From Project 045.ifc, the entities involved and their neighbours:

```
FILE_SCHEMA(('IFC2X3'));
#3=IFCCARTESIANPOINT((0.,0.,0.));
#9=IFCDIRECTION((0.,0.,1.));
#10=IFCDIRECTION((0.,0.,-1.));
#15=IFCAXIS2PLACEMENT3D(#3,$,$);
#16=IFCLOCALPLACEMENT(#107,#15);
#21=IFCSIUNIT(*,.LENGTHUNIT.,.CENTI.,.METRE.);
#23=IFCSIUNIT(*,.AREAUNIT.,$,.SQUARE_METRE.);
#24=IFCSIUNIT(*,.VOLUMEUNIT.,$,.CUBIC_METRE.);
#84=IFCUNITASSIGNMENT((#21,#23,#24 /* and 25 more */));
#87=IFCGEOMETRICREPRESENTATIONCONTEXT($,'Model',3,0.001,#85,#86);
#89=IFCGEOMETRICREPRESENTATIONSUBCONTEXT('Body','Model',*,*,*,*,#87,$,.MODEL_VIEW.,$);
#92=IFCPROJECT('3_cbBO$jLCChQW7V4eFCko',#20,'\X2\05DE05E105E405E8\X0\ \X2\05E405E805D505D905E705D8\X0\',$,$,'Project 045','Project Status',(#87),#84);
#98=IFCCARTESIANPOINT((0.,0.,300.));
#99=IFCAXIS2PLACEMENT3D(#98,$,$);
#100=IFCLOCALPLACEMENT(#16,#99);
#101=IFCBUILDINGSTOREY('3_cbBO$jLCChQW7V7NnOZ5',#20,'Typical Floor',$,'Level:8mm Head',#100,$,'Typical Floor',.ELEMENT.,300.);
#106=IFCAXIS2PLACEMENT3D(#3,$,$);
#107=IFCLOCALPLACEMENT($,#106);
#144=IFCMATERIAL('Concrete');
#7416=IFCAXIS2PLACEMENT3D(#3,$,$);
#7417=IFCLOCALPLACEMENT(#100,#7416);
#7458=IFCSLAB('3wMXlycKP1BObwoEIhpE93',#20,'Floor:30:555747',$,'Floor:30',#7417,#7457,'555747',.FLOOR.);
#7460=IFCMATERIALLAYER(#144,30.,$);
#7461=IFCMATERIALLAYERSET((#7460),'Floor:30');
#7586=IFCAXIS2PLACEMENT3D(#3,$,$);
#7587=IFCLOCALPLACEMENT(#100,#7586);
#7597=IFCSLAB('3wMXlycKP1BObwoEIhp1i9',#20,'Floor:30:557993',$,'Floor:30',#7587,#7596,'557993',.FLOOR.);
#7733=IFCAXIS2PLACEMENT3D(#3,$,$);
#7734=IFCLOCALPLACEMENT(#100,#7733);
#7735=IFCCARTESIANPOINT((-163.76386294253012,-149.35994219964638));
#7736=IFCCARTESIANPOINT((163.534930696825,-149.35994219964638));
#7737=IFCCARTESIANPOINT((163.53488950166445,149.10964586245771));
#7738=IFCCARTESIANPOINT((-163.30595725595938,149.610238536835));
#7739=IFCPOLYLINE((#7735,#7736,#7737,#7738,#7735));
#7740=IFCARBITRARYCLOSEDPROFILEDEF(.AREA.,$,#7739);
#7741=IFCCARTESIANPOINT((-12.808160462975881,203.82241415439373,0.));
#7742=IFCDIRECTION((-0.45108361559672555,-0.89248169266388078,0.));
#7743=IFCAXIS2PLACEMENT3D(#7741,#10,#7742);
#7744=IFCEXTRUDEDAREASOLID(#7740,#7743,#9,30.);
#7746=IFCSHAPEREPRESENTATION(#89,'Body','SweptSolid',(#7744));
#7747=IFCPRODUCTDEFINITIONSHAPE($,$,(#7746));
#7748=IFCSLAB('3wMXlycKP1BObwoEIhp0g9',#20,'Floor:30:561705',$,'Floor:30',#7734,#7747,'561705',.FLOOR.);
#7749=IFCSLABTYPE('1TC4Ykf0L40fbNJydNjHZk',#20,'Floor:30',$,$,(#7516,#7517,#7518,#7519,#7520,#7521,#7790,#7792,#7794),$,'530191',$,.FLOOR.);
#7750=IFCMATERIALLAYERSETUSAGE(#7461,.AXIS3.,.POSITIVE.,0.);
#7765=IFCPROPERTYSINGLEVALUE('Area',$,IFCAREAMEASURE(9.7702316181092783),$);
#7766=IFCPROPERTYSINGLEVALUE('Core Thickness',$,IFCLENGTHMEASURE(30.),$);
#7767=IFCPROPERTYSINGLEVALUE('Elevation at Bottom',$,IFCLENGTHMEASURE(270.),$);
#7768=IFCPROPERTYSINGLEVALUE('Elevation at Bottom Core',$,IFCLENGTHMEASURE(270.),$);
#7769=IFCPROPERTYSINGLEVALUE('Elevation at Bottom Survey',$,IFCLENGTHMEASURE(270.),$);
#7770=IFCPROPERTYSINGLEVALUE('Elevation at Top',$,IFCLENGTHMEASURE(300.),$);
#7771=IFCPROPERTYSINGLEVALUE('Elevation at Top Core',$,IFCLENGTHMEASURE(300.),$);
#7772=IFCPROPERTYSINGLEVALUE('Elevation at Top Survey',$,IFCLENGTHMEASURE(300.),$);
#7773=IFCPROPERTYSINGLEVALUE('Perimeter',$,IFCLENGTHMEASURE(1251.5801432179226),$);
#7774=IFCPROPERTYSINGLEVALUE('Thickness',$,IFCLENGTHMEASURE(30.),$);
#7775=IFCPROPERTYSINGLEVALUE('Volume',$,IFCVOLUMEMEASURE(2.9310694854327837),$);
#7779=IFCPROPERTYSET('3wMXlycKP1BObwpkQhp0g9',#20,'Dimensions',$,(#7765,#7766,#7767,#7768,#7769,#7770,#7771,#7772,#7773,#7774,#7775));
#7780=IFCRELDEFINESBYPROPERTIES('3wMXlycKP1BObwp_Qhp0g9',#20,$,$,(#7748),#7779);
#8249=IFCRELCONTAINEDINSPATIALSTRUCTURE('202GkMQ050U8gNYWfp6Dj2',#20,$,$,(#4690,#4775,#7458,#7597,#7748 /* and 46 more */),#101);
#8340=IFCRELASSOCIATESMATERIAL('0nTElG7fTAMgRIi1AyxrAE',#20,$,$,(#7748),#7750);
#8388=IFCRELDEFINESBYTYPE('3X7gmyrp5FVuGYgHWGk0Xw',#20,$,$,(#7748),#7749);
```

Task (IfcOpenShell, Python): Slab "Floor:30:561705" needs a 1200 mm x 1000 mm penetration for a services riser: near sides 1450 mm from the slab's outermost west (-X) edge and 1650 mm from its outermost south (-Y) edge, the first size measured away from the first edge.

```python
import numpy as np
import ifcopenshell
import ifcopenshell.api.feature
import ifcopenshell.api.geometry
import ifcopenshell.api.pset
import ifcopenshell.api.root
import ifcopenshell.geom
import ifcopenshell.util.element
import ifcopenshell.util.placement
import ifcopenshell.util.representation
import ifcopenshell.util.shape
import ifcopenshell.util.unit

model = ifcopenshell.open("Project 045.ifc")
unit_scale = ifcopenshell.util.unit.calculate_unit_scale(model)
area_scale = ifcopenshell.util.unit.calculate_unit_scale(model, "AREAUNIT")
volume_scale = ifcopenshell.util.unit.calculate_unit_scale(model, "VOLUMEUNIT")
settings = ifcopenshell.geom.settings()


def volume(element):
    """Net volume in cubic metres, openings subtracted."""
    shape = ifcopenshell.geom.create_shape(settings, element)
    return ifcopenshell.util.shape.get_volume(shape.geometry)


slab = model.by_guid("3wMXlycKP1BObwoEIhp0g9")
before = volume(slab)

# Extent in the slab's own axes, in metres. The edges named are its -X and -Y sides.
slab_shape = ifcopenshell.geom.create_shape(settings, slab)
vertices = ifcopenshell.util.shape.get_vertices(slab_shape.geometry)
x_min, y_min, bottom = vertices.min(axis=0)
top = vertices[:, 2].max()

opening = ifcopenshell.api.root.create_entity(model, ifc_class="IfcOpeningElement", name="Services riser opening")
context = ifcopenshell.util.representation.get_context(model, "Model", "Body", "MODEL_VIEW")
width, depth = 1.2, 1
outline = [(0.0, 0.0), (width, 0.0), (width, depth), (0.0, depth), (0.0, 0.0)]
# Overshoot both faces by 50 mm so the cut is clean.
shape = ifcopenshell.api.geometry.add_slab_representation(
    model, context=context, depth=top - bottom + 0.1, polyline=outline
)
ifcopenshell.api.geometry.assign_representation(model, product=opening, representation=shape)

matrix = ifcopenshell.util.placement.get_local_placement(slab.ObjectPlacement)
matrix[:, 3] = matrix @ np.append(np.array([x_min + 1.45, y_min + 1.65, bottom - 0.05]) / unit_scale, 1.0)
ifcopenshell.api.geometry.edit_object_placement(model, product=opening, matrix=matrix, is_si=False)
ifcopenshell.api.feature.add_feature(model, feature=opening, element=slab)

after = volume(slab)

# Update the slab's stored quantities.
pset = model.by_id(ifcopenshell.util.element.get_pset(slab, "Dimensions", should_inherit=False)["id"])
ifcopenshell.api.pset.edit_pset(model, pset=pset, properties={
    "Area": model.create_entity("IfcAreaMeasure", after / (top - bottom) / area_scale),
    "Volume": model.create_entity("IfcVolumeMeasure", after / volume_scale),
})

print(f"slab volume {before:.3f} -> {after:.3f} m3")

model.write("Project 045_rev.ifc")
```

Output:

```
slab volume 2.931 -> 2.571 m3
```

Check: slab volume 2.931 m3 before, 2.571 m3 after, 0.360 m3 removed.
